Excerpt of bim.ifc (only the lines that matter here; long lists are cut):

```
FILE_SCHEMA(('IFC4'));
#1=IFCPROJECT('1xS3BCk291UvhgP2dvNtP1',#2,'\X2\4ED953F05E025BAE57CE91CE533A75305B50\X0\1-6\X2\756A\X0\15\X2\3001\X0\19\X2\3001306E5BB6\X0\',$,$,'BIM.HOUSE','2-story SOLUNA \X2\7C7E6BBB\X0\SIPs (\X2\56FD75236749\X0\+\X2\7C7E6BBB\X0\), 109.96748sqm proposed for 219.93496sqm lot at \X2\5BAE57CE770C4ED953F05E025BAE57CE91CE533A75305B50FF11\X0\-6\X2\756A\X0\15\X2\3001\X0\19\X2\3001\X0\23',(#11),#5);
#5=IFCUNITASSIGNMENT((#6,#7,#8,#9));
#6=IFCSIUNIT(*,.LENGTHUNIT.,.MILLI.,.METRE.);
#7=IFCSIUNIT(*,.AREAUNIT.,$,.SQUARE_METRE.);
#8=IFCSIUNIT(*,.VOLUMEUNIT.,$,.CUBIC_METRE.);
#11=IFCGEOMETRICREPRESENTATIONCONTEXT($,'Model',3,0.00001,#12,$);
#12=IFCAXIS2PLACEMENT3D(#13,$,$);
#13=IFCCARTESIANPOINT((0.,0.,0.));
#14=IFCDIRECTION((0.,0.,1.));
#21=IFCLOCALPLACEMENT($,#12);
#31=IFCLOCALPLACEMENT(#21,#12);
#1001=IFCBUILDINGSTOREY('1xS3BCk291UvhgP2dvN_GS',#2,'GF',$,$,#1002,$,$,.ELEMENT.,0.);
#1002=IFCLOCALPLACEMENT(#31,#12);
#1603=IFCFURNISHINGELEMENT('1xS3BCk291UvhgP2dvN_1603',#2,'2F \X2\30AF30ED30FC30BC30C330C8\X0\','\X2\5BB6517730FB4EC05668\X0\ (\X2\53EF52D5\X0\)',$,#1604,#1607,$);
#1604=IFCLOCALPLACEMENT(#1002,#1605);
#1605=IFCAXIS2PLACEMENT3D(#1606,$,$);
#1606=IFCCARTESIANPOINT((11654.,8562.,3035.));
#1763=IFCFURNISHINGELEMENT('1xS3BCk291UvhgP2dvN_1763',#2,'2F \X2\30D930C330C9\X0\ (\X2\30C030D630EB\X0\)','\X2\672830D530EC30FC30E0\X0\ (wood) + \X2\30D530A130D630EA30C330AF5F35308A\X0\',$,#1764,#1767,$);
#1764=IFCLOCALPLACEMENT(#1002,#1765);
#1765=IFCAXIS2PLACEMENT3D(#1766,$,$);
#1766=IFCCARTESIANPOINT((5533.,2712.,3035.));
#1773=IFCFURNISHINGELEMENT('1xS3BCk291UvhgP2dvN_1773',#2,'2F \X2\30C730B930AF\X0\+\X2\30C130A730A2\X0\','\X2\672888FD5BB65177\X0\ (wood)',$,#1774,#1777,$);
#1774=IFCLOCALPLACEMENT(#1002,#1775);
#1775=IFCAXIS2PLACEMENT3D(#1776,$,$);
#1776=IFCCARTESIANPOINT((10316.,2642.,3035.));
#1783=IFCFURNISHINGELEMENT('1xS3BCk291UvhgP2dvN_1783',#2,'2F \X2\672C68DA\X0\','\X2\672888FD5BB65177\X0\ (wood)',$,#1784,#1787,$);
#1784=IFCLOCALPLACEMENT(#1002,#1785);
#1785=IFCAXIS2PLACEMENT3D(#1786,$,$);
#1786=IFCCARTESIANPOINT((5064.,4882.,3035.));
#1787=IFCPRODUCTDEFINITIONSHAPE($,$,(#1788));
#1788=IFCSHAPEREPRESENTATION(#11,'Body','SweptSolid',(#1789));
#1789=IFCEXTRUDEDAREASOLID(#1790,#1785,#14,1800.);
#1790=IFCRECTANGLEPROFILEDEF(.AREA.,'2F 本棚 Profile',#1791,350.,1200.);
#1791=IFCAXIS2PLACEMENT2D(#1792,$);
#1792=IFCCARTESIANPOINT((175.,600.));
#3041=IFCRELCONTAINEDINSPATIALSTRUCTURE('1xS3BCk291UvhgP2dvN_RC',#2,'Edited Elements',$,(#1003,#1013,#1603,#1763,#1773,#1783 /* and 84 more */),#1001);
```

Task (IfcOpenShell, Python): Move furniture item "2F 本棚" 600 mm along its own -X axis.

```python
import ifcopenshell
import ifcopenshell.api.geometry
import ifcopenshell.util.placement

model = ifcopenshell.open("bim.ifc")

item = model.by_guid("1xS3BCk291UvhgP2dvN_1783")
matrix = ifcopenshell.util.placement.get_local_placement(item.ObjectPlacement)
matrix[:3, 3] -= matrix[:3, 0] * 600.0
ifcopenshell.api.geometry.edit_object_placement(model, product=item, matrix=matrix, is_si=False)

print(ifcopenshell.util.placement.get_local_placement(item.ObjectPlacement).round(3) + 0.0)

model.write("bim_updated.ifc")
```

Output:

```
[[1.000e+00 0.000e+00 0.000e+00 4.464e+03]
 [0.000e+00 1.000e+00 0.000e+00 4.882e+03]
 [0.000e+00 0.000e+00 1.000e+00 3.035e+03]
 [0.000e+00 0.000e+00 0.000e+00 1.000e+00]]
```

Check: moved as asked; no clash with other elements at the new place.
